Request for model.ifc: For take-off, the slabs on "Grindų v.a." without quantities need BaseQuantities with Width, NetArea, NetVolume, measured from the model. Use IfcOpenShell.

First a look at what the model holds.

```python
import ifcopenshell
import ifcopenshell.util.element
import ifcopenshell.util.unit

model = ifcopenshell.open("model.ifc")
print(model.schema)
for unit_type in ("LENGTHUNIT", "AREAUNIT", "VOLUMEUNIT"):
    print(unit_type, ifcopenshell.util.unit.calculate_unit_scale(model, unit_type))
storey = next(s for s in model.by_type("IfcBuildingStorey") if s.Name == "Grindų v.a.")
slabs = [e for e in ifcopenshell.util.element.get_decomposition(storey) if e.is_a("IfcSlab")]
for e in sorted(slabs, key=lambda e: e.id()):
    print(e.id(), e.is_a(), e.Name, list(ifcopenshell.util.element.get_psets(e, qtos_only=True)), sep=" | ")
```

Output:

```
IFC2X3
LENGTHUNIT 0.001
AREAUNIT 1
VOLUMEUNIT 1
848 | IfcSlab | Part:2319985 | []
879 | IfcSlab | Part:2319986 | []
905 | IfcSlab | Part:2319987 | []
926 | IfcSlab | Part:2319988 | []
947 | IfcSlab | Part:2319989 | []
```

```python
import ifcopenshell
import ifcopenshell.api.pset
import ifcopenshell.geom
import ifcopenshell.util.element
import ifcopenshell.util.shape
import ifcopenshell.util.unit

model = ifcopenshell.open("model.ifc")
unit_scale = ifcopenshell.util.unit.calculate_unit_scale(model)
area_scale = ifcopenshell.util.unit.calculate_unit_scale(model, "AREAUNIT")
volume_scale = ifcopenshell.util.unit.calculate_unit_scale(model, "VOLUMEUNIT")
settings = ifcopenshell.geom.settings()

storey = next(s for s in model.by_type("IfcBuildingStorey") if s.Name == "Grindų v.a.")
slabs = [e for e in ifcopenshell.util.element.get_decomposition(storey) if e.is_a("IfcSlab")]

for e in sorted(slabs, key=lambda e: e.id()):
    if ifcopenshell.util.element.get_psets(e, qtos_only=True, should_inherit=False):
        continue
    # Geometry comes back in metres, in the element's own axes.
    shape = ifcopenshell.geom.create_shape(settings, e)
    values = {
        "Width": ifcopenshell.util.shape.get_z(shape.geometry) / unit_scale,
        "NetArea": ifcopenshell.util.shape.get_footprint_area(shape.geometry) / area_scale,
        "NetVolume": ifcopenshell.util.shape.get_volume(shape.geometry) / volume_scale,
    }
    qto = ifcopenshell.api.pset.add_qto(model, product=e, name="BaseQuantities")
    ifcopenshell.api.pset.edit_qto(model, qto=qto, properties=values)
    print(e.id(), {k: round(v, 3) for k, v in values.items()})

model.write("model-out.ifc")
```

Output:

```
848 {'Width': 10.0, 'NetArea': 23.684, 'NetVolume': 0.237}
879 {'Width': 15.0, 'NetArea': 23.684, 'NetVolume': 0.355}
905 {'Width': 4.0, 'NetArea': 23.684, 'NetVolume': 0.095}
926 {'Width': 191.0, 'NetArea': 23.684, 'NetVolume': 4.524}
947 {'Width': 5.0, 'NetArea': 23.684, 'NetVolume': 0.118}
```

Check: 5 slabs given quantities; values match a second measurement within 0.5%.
